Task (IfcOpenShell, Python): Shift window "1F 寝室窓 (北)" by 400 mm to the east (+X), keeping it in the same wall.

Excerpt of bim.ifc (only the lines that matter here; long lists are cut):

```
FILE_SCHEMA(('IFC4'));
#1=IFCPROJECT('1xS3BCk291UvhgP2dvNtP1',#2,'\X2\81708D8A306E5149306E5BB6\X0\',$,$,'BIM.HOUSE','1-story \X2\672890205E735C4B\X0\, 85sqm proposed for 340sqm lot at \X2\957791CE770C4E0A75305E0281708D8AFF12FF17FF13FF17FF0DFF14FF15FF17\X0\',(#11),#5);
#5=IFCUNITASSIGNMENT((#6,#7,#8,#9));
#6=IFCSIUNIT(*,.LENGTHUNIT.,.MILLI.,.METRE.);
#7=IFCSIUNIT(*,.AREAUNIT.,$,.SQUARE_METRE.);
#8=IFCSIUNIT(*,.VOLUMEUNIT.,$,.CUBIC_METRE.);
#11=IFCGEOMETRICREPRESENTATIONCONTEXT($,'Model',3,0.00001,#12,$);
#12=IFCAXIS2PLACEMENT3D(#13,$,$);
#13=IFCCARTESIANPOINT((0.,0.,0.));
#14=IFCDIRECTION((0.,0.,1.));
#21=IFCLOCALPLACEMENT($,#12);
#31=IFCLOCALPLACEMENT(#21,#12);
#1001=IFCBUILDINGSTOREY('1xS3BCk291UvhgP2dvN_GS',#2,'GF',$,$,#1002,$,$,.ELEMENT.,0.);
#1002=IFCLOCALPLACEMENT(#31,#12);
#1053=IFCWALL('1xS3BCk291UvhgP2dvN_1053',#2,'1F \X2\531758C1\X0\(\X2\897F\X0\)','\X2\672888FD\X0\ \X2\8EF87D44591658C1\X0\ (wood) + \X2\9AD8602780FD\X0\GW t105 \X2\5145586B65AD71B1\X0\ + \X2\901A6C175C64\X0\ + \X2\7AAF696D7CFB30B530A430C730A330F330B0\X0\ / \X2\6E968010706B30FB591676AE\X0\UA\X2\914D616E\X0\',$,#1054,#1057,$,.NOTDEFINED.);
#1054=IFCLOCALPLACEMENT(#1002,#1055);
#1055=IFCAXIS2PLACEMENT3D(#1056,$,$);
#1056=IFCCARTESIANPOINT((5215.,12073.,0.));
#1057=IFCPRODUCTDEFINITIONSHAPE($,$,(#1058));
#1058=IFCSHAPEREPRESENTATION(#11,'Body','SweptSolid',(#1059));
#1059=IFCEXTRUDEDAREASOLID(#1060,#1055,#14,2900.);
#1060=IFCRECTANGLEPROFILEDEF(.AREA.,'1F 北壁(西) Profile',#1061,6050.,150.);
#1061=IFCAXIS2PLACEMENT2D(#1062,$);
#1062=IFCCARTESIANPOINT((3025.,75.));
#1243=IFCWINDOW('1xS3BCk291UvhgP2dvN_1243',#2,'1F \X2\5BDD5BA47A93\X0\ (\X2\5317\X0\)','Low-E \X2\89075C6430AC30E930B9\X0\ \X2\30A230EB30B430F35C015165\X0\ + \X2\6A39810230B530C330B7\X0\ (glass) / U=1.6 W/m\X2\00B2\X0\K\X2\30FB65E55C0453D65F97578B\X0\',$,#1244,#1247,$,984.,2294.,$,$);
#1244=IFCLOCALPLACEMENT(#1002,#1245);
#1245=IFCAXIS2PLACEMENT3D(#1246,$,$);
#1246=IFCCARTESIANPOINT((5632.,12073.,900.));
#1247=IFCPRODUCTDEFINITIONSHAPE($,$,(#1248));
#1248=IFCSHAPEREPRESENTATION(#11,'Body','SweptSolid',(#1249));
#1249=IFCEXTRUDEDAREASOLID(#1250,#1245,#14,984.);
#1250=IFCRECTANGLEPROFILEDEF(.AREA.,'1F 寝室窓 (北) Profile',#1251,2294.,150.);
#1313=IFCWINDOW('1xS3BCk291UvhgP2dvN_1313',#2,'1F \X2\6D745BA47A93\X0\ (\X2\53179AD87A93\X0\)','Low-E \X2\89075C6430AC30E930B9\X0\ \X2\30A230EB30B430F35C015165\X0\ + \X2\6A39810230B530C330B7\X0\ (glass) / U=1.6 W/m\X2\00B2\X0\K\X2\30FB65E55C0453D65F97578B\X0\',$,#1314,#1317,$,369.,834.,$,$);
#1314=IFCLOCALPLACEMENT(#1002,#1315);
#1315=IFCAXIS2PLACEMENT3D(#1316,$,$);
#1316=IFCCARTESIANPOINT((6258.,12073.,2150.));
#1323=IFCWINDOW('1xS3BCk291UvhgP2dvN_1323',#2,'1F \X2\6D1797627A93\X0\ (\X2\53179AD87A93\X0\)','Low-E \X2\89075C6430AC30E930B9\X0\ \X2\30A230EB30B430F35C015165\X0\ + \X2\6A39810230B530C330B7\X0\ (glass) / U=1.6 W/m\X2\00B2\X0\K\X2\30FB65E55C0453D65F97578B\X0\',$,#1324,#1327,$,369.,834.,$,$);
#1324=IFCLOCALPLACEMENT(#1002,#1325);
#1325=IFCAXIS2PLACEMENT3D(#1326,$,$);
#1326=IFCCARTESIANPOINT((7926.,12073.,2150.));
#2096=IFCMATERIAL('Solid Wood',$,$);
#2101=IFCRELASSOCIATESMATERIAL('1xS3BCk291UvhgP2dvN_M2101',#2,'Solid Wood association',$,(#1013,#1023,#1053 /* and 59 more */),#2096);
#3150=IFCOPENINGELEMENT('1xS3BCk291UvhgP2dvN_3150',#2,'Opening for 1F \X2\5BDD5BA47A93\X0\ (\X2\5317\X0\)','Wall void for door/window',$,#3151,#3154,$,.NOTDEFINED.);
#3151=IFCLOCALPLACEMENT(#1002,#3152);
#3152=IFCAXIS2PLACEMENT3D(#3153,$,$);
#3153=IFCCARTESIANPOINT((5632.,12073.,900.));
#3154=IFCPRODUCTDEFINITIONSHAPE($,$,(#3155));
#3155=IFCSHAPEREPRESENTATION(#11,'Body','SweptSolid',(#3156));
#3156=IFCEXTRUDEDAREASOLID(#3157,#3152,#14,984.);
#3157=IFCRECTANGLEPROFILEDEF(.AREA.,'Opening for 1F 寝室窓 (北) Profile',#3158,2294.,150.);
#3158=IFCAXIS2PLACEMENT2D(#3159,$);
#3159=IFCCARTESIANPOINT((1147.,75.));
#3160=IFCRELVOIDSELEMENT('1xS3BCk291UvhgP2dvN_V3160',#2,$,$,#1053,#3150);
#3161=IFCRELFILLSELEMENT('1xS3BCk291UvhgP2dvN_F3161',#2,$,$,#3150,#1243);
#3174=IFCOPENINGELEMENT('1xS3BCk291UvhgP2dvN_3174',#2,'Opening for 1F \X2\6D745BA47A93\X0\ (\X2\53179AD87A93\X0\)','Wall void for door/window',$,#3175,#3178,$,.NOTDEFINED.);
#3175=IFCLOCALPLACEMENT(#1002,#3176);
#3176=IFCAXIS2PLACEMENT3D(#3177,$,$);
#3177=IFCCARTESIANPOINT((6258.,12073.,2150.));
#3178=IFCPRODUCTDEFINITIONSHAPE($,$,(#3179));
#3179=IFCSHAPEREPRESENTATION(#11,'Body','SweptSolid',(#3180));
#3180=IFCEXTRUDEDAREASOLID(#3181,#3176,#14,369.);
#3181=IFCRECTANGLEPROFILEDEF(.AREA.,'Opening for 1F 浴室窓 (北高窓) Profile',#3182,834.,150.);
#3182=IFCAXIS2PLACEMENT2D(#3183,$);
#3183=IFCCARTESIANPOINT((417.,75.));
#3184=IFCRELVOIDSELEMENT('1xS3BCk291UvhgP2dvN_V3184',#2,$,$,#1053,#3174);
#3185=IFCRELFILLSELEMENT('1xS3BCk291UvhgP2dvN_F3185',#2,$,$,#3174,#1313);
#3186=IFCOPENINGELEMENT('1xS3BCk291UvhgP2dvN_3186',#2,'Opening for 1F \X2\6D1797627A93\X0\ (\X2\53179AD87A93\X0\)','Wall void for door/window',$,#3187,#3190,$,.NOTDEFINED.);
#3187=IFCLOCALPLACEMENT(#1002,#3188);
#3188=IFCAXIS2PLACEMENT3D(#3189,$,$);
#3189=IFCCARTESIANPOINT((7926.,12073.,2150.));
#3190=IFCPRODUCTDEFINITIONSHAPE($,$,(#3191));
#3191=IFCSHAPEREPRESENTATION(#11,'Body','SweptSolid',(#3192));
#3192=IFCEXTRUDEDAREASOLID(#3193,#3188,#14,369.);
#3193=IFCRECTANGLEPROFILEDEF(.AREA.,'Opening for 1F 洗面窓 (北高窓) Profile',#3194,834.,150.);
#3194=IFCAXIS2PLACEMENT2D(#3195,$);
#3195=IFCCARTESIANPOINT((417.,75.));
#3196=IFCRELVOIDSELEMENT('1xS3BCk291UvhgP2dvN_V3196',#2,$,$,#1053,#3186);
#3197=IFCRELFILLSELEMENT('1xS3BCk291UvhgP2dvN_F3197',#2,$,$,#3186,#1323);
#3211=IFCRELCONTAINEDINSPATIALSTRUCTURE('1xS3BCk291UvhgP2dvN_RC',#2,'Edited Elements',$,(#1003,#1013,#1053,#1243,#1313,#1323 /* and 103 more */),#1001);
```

```python
import ifcopenshell
import ifcopenshell.api.geometry
import ifcopenshell.util.placement

model = ifcopenshell.open("bim.ifc")

window = model.by_guid("1xS3BCk291UvhgP2dvN_1243")
opening = window.FillsVoids[0].RelatingOpeningElement
wall = opening.VoidsElements[0].RelatingBuildingElement

wall_matrix = ifcopenshell.util.placement.get_local_placement(wall.ObjectPlacement)
shift = wall_matrix[:3, 0] * 400.0
before = ifcopenshell.util.placement.get_local_placement(window.ObjectPlacement)[:3, 3].copy()

# The window is not placed relative to its opening, so move both.
for product in (opening, window):
    matrix = ifcopenshell.util.placement.get_local_placement(product.ObjectPlacement)
    matrix[:3, 3] += shift
    ifcopenshell.api.geometry.edit_object_placement(model, product=product, matrix=matrix, is_si=False)

after = ifcopenshell.util.placement.get_local_placement(window.ObjectPlacement)[:3, 3]
print("window moved by", (after - before).round(3) + 0.0)

model.write("bim_edited.ifc")
```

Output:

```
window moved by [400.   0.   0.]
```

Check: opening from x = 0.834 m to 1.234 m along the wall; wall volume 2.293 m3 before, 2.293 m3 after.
